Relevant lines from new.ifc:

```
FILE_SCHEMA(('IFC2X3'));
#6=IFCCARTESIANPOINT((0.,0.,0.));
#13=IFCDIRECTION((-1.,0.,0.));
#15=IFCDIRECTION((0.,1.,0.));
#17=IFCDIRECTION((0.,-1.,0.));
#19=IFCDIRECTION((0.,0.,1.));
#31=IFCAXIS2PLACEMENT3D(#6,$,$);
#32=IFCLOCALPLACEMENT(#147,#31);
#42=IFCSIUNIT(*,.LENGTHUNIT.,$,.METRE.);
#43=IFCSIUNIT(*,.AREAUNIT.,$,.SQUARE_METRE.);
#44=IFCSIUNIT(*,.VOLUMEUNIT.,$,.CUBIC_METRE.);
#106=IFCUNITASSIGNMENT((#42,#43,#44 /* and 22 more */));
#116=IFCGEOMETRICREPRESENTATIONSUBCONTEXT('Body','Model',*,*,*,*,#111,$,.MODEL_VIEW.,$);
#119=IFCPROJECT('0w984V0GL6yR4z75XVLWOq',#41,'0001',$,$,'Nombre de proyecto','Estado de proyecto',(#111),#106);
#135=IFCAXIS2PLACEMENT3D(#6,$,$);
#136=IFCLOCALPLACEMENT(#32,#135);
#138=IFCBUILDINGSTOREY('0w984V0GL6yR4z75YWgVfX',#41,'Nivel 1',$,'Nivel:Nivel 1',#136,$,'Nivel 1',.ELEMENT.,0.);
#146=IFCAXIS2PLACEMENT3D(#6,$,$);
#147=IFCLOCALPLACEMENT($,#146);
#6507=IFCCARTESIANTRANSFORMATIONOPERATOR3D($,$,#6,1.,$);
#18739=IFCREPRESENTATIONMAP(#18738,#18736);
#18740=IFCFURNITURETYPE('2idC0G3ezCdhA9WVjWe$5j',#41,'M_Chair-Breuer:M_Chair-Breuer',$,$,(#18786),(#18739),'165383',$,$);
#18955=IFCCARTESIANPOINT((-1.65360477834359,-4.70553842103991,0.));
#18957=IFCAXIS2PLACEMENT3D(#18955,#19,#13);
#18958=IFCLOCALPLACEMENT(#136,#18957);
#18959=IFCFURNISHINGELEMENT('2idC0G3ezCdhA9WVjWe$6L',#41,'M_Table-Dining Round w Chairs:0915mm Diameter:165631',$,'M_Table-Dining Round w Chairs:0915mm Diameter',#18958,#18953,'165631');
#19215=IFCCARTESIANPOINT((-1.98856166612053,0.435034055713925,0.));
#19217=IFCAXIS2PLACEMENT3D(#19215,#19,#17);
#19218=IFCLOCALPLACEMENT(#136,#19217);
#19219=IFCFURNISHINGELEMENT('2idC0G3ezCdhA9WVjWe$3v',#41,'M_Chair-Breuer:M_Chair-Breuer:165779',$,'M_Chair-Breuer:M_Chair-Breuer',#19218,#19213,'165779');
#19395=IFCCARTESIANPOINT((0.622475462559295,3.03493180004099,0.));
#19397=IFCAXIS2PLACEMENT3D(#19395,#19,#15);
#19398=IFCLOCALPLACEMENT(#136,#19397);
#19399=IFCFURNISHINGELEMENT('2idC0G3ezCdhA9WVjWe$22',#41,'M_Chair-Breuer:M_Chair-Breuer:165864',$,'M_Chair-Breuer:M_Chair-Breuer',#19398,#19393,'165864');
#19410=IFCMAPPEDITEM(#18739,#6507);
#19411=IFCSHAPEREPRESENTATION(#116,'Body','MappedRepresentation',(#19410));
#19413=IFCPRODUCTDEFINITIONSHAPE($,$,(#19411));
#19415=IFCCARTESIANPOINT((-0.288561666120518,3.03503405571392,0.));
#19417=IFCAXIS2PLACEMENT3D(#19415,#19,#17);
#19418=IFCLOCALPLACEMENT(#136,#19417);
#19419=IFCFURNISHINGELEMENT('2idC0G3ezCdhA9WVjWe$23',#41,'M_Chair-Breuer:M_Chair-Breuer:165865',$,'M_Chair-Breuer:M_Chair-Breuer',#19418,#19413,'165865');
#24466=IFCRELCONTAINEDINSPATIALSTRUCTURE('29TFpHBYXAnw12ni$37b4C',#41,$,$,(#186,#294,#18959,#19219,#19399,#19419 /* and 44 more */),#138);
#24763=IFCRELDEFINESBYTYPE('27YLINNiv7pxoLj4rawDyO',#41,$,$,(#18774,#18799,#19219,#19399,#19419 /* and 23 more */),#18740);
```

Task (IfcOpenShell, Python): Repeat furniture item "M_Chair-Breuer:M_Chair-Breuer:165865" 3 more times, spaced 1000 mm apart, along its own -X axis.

```python
import ifcopenshell
import ifcopenshell.api.geometry
import ifcopenshell.api.root
import ifcopenshell.util.element
import ifcopenshell.util.placement
import ifcopenshell.util.unit

model = ifcopenshell.open("new.ifc")
unit_scale = ifcopenshell.util.unit.calculate_unit_scale(model)


def reuse_history(source, copy):
    """copy_class also copies each property set's owner history, people and application; keep the originals."""
    for rel in copy.IsDefinedBy:
        if rel.is_a("IfcRelDefinesByProperties") and (history := rel.RelatingPropertyDefinition.OwnerHistory):
            rel.RelatingPropertyDefinition.OwnerHistory = source.OwnerHistory
            ifcopenshell.util.element.remove_deep2(model, history)


source = model.by_id(19419)
base = ifcopenshell.util.placement.get_local_placement(source.ObjectPlacement)
step = -base[:3, 0] * 1 / unit_scale

for i in range(1, 4):
    copy = ifcopenshell.api.root.copy_class(model, product=source)
    copy.Representation = ifcopenshell.util.element.copy_deep(
        model, source.Representation, exclude=["IfcGeometricRepresentationContext", "IfcRepresentationMap"]
    )
    copy.Name = "M_Chair-Breuer:M_Chair-Breuer"
    copy.Tag = None
    reuse_history(source, copy)
    matrix = base.copy()
    matrix[:3, 3] += i * step
    print("added at", matrix[:3, 3].round(3) + 0.0)
    ifcopenshell.api.geometry.edit_object_placement(model, product=copy, matrix=matrix, is_si=False)

model.write("new_edited.ifc")
```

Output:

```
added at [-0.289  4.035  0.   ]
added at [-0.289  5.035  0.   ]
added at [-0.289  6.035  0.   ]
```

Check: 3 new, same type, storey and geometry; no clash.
